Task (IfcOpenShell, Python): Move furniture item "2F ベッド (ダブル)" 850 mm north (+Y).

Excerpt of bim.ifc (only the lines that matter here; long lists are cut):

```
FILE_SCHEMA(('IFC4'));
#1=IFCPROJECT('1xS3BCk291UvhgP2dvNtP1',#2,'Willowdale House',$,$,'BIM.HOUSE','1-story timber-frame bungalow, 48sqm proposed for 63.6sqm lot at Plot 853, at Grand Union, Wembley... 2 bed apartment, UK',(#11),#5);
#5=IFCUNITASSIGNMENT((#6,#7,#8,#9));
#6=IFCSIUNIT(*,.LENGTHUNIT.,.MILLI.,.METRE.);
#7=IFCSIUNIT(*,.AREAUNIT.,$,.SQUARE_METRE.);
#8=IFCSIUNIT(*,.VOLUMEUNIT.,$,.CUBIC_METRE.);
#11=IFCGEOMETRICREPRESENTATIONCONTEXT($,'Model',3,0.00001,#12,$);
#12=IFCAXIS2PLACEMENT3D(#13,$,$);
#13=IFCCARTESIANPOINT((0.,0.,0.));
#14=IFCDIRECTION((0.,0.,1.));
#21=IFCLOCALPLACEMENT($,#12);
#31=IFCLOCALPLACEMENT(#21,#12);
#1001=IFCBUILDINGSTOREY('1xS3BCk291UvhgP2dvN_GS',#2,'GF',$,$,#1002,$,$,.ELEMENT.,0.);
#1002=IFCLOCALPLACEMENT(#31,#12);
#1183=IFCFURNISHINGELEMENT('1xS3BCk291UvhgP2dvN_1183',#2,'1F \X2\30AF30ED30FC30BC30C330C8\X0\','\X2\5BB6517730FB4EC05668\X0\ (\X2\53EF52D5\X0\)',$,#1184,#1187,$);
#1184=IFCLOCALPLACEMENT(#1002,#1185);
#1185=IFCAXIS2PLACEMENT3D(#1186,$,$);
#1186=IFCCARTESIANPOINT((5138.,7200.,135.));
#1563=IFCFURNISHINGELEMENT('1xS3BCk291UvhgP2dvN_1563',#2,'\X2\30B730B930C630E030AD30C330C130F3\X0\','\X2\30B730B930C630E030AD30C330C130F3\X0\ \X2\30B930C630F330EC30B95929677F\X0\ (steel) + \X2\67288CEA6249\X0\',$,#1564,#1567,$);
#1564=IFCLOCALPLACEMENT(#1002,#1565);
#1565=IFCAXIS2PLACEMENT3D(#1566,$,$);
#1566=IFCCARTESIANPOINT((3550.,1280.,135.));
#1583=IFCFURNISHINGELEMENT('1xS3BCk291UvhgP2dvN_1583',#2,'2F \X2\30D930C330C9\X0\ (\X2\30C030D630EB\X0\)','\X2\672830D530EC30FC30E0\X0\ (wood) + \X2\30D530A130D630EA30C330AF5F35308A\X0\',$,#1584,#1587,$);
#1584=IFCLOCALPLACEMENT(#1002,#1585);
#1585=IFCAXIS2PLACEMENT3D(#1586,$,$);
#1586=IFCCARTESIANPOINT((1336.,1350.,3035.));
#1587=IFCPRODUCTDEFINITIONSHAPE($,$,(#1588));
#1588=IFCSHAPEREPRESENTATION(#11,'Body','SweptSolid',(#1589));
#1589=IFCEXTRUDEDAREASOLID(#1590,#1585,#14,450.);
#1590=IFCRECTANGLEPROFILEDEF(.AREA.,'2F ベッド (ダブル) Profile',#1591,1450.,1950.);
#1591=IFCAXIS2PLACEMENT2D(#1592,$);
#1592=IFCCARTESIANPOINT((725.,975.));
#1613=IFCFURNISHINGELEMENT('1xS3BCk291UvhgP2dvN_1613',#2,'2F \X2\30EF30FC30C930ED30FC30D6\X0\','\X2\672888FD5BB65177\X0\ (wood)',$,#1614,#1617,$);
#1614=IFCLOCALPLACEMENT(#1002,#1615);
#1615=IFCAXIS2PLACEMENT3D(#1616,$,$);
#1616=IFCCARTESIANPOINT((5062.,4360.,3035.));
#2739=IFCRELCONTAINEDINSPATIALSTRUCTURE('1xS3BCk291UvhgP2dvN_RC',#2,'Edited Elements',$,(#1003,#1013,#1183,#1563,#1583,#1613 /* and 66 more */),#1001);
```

```python
import ifcopenshell
import ifcopenshell.api.geometry
import ifcopenshell.util.placement

model = ifcopenshell.open("bim.ifc")

item = model.by_id(1583)
matrix = ifcopenshell.util.placement.get_local_placement(item.ObjectPlacement)
matrix[1, 3] += 850.0
ifcopenshell.api.geometry.edit_object_placement(model, product=item, matrix=matrix, is_si=False)

print(ifcopenshell.util.placement.get_local_placement(item.ObjectPlacement).round(3) + 0.0)

model.write("bim_edited.ifc")
```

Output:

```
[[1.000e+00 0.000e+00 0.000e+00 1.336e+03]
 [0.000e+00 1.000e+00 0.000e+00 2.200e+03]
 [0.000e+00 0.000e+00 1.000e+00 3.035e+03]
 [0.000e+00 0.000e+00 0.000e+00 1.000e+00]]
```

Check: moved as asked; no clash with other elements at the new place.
